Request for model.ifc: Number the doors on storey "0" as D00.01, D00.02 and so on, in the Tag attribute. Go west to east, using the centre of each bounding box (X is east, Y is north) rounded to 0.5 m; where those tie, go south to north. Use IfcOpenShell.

First a look at what the model holds.

```python
import ifcopenshell
import ifcopenshell.util.element
import ifcopenshell.util.placement

model = ifcopenshell.open("model.ifc")
print(model.schema)
storey = next(s for s in model.by_type("IfcBuildingStorey") if s.Name == "0")
doors = [e for e in ifcopenshell.util.element.get_decomposition(storey) if e.is_a("IfcDoor")]
for e in sorted(doors, key=lambda e: e.id()):
    origin = ifcopenshell.util.placement.get_local_placement(e.ObjectPlacement)[:3, 3]
    print(e.id(), e.Tag, e.Name, origin.round(2) + 0.0, sep=" | ")
```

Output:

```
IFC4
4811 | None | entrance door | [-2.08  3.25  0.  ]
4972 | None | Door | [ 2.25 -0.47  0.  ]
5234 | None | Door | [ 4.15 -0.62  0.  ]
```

```python
import ifcopenshell
import ifcopenshell.geom
import ifcopenshell.util.element
import ifcopenshell.util.shape

model = ifcopenshell.open("model.ifc")
settings = ifcopenshell.geom.settings()
settings.set("use-world-coords", True)


def centre(element):
    shape = ifcopenshell.geom.create_shape(settings, element)
    return ifcopenshell.util.shape.get_bbox_centroid(shape.geometry)


storey = next(s for s in model.by_type("IfcBuildingStorey") if s.Name == "0")
doors = [e for e in ifcopenshell.util.element.get_decomposition(storey) if e.is_a("IfcDoor")]

# Insertion points can sit at a corner or the storey origin, so sort by the geometry (in metres).
centres = {e: centre(e) for e in doors}
doors.sort(key=lambda e: (round(centres[e][0] / 0.5), centres[e][1]))

for i, e in enumerate(doors, start=1):
    number = f"D00.{i:02d}"
    e.Tag = number
    print(e.id(), number)

model.write("model_edited.ifc")
```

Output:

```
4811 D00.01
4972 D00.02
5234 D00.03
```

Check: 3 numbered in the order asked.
